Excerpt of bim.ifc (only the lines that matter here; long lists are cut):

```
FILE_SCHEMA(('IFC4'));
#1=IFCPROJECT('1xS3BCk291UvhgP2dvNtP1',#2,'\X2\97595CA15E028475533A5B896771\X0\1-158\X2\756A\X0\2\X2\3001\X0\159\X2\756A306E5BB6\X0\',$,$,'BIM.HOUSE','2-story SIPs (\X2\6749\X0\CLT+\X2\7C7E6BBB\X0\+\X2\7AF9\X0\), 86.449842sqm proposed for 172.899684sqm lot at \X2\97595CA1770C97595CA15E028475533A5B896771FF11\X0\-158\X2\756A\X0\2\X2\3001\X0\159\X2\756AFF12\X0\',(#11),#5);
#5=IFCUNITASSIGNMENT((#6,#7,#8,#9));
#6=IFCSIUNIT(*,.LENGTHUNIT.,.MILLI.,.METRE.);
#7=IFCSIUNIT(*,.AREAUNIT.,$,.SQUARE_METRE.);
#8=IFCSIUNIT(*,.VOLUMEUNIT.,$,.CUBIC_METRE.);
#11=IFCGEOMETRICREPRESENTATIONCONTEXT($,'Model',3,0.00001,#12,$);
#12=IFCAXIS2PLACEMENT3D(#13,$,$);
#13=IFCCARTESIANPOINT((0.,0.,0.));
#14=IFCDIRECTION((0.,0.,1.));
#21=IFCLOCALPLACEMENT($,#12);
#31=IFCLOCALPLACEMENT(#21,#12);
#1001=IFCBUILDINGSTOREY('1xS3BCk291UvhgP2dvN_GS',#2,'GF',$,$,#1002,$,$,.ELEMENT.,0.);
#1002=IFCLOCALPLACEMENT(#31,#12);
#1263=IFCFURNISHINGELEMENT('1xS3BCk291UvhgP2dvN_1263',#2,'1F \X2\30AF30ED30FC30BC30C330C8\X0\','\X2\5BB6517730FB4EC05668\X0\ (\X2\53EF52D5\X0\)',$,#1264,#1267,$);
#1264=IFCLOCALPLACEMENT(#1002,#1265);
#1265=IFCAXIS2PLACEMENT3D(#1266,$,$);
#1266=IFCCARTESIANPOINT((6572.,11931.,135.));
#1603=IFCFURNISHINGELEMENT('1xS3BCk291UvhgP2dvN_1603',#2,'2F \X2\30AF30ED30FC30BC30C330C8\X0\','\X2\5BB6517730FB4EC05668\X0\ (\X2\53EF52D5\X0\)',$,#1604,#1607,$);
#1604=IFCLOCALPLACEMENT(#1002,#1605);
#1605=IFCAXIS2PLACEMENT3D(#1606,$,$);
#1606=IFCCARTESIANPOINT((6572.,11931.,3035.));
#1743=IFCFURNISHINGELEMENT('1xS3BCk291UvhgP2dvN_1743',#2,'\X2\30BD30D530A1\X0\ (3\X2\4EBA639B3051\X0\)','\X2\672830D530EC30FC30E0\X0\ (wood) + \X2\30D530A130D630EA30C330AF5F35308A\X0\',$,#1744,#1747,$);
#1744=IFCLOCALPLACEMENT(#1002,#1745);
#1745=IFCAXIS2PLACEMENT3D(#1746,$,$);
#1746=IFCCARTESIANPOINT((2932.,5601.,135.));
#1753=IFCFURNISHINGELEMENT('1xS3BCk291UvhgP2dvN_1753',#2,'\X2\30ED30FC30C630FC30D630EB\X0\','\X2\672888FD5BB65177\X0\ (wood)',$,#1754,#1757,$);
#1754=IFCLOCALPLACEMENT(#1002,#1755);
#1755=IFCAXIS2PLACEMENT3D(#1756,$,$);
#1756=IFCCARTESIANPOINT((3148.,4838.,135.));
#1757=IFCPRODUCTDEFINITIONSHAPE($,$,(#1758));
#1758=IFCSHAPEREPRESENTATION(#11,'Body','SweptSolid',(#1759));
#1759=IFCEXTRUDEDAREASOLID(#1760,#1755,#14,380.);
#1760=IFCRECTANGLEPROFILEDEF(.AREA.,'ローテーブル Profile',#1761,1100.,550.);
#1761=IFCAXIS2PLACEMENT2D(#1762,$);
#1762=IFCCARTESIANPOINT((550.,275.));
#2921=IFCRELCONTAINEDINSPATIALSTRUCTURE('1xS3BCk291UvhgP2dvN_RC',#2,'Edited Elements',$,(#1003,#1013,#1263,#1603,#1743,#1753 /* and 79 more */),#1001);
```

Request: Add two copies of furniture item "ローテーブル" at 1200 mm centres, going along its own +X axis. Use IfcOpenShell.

```python
import ifcopenshell
import ifcopenshell.api.geometry
import ifcopenshell.api.root
import ifcopenshell.util.element
import ifcopenshell.util.placement
import ifcopenshell.util.unit

model = ifcopenshell.open("bim.ifc")
unit_scale = ifcopenshell.util.unit.calculate_unit_scale(model)


def reuse_history(source, copy):
    """copy_class also copies each property set's owner history, people and application; keep the originals."""
    for rel in copy.IsDefinedBy:
        if rel.is_a("IfcRelDefinesByProperties") and (history := rel.RelatingPropertyDefinition.OwnerHistory):
            rel.RelatingPropertyDefinition.OwnerHistory = source.OwnerHistory
            ifcopenshell.util.element.remove_deep2(model, history)


source = model.by_guid("1xS3BCk291UvhgP2dvN_1753")
base = ifcopenshell.util.placement.get_local_placement(source.ObjectPlacement)
step = base[:3, 0] * 1.2 / unit_scale

for i in range(1, 3):
    copy = ifcopenshell.api.root.copy_class(model, product=source)
    copy.Representation = ifcopenshell.util.element.copy_deep(
        model, source.Representation, exclude=["IfcGeometricRepresentationContext", "IfcRepresentationMap"]
    )
    reuse_history(source, copy)
    matrix = base.copy()
    matrix[:3, 3] += i * step
    print("added at", matrix[:3, 3].round(3) + 0.0)
    ifcopenshell.api.geometry.edit_object_placement(model, product=copy, matrix=matrix, is_si=False)

model.write("bim_updated.ifc")
```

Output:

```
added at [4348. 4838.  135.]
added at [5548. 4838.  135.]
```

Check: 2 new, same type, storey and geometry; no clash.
